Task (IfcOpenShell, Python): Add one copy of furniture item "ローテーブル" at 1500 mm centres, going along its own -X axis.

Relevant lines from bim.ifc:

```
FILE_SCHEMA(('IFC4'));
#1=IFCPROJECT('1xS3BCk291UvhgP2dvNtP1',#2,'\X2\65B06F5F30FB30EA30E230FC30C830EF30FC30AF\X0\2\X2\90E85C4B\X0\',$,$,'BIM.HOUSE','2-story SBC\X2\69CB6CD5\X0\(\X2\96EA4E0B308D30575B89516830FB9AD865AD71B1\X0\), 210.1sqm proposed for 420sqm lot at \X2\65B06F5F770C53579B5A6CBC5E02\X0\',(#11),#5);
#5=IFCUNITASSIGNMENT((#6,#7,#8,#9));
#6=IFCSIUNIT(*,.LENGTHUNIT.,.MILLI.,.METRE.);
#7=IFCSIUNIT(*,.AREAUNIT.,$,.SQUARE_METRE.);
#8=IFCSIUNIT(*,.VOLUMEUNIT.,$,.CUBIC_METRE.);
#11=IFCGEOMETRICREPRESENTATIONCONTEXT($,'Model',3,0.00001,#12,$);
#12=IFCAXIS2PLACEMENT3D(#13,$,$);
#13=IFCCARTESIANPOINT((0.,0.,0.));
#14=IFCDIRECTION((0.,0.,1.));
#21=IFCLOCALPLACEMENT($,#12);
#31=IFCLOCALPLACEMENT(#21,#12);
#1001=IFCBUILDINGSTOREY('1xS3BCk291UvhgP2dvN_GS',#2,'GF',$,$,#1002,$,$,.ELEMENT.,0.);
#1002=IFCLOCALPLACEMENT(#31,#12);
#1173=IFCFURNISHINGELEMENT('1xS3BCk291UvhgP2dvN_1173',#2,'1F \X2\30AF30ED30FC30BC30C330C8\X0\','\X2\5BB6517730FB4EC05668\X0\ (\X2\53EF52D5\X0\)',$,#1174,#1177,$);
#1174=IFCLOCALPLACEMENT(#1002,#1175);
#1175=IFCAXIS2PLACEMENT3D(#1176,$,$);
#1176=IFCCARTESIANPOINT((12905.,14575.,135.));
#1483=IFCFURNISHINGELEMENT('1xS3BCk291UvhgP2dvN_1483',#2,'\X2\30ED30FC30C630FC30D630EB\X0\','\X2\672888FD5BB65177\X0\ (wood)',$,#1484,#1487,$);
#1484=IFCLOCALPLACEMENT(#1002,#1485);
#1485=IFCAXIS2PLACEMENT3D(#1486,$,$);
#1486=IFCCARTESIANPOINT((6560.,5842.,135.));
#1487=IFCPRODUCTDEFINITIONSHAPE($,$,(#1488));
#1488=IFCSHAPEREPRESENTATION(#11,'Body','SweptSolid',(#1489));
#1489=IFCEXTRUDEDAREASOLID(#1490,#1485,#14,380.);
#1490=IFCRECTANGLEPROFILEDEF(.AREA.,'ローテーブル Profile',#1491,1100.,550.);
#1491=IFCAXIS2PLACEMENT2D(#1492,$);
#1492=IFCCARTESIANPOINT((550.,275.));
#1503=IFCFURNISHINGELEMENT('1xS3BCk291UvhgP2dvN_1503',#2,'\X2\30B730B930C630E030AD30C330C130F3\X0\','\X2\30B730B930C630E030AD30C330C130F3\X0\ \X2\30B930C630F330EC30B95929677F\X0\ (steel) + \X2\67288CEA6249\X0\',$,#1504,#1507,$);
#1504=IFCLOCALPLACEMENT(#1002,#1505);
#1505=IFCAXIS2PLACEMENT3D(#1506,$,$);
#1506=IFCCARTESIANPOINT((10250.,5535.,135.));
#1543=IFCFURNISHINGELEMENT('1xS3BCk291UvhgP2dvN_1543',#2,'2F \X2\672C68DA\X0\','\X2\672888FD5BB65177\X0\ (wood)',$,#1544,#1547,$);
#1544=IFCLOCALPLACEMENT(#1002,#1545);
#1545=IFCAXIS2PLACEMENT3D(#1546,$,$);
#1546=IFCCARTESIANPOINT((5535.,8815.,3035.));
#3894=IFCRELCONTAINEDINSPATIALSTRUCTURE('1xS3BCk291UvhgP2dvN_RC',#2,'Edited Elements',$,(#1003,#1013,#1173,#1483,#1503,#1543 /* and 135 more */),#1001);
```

```python
import ifcopenshell
import ifcopenshell.api.geometry
import ifcopenshell.api.root
import ifcopenshell.util.element
import ifcopenshell.util.placement
import ifcopenshell.util.unit

model = ifcopenshell.open("bim.ifc")
unit_scale = ifcopenshell.util.unit.calculate_unit_scale(model)


def reuse_history(source, copy):
    """copy_class also copies each property set's owner history, people and application; keep the originals."""
    for rel in copy.IsDefinedBy:
        if rel.is_a("IfcRelDefinesByProperties") and (history := rel.RelatingPropertyDefinition.OwnerHistory):
            rel.RelatingPropertyDefinition.OwnerHistory = source.OwnerHistory
            ifcopenshell.util.element.remove_deep2(model, history)


source = model.by_guid("1xS3BCk291UvhgP2dvN_1483")
base = ifcopenshell.util.placement.get_local_placement(source.ObjectPlacement)
step = -base[:3, 0] * 1.5 / unit_scale

for i in range(1, 2):
    copy = ifcopenshell.api.root.copy_class(model, product=source)
    copy.Representation = ifcopenshell.util.element.copy_deep(
        model, source.Representation, exclude=["IfcGeometricRepresentationContext", "IfcRepresentationMap"]
    )
    reuse_history(source, copy)
    matrix = base.copy()
    matrix[:3, 3] += i * step
    print("added at", matrix[:3, 3].round(3) + 0.0)
    ifcopenshell.api.geometry.edit_object_placement(model, product=copy, matrix=matrix, is_si=False)

model.write("bim_edited.ifc")
```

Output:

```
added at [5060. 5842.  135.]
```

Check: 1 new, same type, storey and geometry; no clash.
